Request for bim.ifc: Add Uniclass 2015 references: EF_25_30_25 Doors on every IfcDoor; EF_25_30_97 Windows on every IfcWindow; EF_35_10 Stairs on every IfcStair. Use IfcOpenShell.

First a look at what the model holds.

```python
import ifcopenshell

model = ifcopenshell.open("bim.ifc")
print(model.schema)
print("classifications:", [c.Name for c in model.by_type("IfcClassification")])
for ifc_class in ("IfcDoor", "IfcRoof", "IfcStair", "IfcWall", "IfcWindow"):
    print(ifc_class, len(model.by_type(ifc_class)))
```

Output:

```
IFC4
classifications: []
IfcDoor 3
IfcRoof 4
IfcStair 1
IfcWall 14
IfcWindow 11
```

```python
import ifcopenshell
import ifcopenshell.api.classification

model = ifcopenshell.open("bim.ifc")

system = ifcopenshell.api.classification.add_classification(model, classification="Uniclass 2015")

codes = {
    "IfcDoor": ("EF_25_30_25", "Doors"),
    "IfcWindow": ("EF_25_30_97", "Windows"),
    "IfcStair": ("EF_35_10", "Stairs"),
}
for ifc_class, (code, name) in codes.items():
    products = model.by_type(ifc_class)
    ifcopenshell.api.classification.add_reference(
        model, products=products, classification=system, identification=code, name=name
    )
    print(code, len(products))

model.write("bim_updated.ifc")
```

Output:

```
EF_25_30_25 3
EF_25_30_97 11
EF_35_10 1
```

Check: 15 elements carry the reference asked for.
